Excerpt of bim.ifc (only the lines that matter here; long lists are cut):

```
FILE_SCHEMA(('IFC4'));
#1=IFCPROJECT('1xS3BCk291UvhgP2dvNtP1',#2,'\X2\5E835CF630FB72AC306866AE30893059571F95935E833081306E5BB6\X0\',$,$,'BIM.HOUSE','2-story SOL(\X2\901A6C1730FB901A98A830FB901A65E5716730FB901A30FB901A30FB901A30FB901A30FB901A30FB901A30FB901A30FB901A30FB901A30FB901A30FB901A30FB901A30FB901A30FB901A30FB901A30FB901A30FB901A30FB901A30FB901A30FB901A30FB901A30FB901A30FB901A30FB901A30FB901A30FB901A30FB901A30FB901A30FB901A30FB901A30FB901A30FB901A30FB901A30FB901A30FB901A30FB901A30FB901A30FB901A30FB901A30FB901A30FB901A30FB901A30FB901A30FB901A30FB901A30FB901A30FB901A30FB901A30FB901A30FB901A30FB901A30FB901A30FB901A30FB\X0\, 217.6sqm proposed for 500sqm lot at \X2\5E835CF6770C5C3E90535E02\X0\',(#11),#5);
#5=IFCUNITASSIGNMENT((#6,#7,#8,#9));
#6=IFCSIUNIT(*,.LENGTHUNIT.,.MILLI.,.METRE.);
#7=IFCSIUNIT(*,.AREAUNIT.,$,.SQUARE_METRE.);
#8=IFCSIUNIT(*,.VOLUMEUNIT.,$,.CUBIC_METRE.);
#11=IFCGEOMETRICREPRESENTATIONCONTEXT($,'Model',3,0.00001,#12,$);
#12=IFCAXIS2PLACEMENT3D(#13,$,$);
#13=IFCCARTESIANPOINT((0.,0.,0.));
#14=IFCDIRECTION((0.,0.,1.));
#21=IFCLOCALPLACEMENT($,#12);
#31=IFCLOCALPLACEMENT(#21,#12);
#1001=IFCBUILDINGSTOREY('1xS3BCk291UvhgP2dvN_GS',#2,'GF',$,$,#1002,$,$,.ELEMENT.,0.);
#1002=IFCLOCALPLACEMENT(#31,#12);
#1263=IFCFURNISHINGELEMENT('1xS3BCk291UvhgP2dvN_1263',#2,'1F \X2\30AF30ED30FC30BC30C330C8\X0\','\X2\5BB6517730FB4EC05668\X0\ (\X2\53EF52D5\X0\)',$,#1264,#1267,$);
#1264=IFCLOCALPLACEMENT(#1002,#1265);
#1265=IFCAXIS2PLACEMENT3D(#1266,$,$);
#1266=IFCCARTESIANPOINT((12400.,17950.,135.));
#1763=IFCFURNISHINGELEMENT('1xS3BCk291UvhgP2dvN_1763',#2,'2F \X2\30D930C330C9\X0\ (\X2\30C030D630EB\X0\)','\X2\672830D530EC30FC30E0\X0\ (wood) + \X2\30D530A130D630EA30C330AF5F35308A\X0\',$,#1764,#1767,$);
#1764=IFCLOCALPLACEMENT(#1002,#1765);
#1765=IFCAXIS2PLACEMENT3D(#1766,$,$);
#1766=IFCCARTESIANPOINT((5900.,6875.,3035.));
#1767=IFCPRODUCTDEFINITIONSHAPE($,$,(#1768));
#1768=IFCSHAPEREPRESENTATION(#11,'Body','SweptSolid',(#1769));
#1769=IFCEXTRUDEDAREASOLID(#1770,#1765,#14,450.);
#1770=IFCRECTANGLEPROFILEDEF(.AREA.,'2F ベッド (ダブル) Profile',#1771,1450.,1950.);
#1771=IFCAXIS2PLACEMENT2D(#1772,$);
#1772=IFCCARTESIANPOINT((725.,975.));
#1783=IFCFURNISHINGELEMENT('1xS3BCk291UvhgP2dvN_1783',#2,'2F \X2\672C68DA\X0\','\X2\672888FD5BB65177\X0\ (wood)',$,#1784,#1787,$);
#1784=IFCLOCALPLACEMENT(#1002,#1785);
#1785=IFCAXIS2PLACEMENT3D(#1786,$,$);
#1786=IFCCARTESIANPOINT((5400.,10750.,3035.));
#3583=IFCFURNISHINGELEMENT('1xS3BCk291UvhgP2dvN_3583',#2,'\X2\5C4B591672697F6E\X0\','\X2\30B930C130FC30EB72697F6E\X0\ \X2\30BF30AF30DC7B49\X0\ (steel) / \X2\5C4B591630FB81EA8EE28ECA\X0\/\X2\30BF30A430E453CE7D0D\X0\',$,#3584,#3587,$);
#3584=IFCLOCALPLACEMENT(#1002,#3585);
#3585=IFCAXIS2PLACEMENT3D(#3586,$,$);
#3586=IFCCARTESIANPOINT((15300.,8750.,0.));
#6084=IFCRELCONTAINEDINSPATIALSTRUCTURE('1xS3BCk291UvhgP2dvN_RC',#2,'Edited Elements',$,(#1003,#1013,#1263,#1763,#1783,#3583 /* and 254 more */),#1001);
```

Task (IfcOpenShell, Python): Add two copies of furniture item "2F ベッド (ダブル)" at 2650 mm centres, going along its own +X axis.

```python
import ifcopenshell
import ifcopenshell.api.geometry
import ifcopenshell.api.root
import ifcopenshell.util.element
import ifcopenshell.util.placement

model = ifcopenshell.open("bim.ifc")


def reuse_history(source, copy):
    """copy_class also copies each property set's owner history, people and application; keep the originals."""
    for rel in copy.IsDefinedBy:
        if rel.is_a("IfcRelDefinesByProperties") and (history := rel.RelatingPropertyDefinition.OwnerHistory):
            rel.RelatingPropertyDefinition.OwnerHistory = source.OwnerHistory
            ifcopenshell.util.element.remove_deep2(model, history)


source = model.by_id(1763)
base = ifcopenshell.util.placement.get_local_placement(source.ObjectPlacement)
step = base[:3, 0] * 2650.0

for i in range(1, 3):
    copy = ifcopenshell.api.root.copy_class(model, product=source)
    copy.Representation = ifcopenshell.util.element.copy_deep(
        model, source.Representation, exclude=["IfcGeometricRepresentationContext", "IfcRepresentationMap"]
    )
    reuse_history(source, copy)
    matrix = base.copy()
    matrix[:3, 3] += i * step
    print("added at", matrix[:3, 3].round(3) + 0.0)
    ifcopenshell.api.geometry.edit_object_placement(model, product=copy, matrix=matrix, is_si=False)

model.write("bim_v2.ifc")
```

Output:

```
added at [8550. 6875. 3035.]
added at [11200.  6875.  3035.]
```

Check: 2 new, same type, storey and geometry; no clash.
